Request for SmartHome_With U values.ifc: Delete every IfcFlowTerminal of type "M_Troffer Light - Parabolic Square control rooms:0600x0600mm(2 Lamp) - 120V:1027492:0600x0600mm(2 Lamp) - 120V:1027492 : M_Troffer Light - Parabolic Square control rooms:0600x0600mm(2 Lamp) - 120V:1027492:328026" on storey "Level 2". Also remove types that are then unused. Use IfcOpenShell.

First a look at what the model holds.

```python
import ifcopenshell
import ifcopenshell.util.element

model = ifcopenshell.open("SmartHome_With U values.ifc")
print(model.schema)
storey = next(s for s in model.by_type("IfcBuildingStorey") if s.Name == "Level 2")
terminals = [e for e in ifcopenshell.util.element.get_decomposition(storey) if e.is_a("IfcFlowTerminal")]
seen = {}
for e in terminals:
    element_type = ifcopenshell.util.element.get_type(e)
    name = element_type.Name if element_type not in (None, e) else None
    seen[name] = seen.get(name, 0) + 1
for name, count in sorted(seen.items(), key=str):
    print(count, "x", name)
```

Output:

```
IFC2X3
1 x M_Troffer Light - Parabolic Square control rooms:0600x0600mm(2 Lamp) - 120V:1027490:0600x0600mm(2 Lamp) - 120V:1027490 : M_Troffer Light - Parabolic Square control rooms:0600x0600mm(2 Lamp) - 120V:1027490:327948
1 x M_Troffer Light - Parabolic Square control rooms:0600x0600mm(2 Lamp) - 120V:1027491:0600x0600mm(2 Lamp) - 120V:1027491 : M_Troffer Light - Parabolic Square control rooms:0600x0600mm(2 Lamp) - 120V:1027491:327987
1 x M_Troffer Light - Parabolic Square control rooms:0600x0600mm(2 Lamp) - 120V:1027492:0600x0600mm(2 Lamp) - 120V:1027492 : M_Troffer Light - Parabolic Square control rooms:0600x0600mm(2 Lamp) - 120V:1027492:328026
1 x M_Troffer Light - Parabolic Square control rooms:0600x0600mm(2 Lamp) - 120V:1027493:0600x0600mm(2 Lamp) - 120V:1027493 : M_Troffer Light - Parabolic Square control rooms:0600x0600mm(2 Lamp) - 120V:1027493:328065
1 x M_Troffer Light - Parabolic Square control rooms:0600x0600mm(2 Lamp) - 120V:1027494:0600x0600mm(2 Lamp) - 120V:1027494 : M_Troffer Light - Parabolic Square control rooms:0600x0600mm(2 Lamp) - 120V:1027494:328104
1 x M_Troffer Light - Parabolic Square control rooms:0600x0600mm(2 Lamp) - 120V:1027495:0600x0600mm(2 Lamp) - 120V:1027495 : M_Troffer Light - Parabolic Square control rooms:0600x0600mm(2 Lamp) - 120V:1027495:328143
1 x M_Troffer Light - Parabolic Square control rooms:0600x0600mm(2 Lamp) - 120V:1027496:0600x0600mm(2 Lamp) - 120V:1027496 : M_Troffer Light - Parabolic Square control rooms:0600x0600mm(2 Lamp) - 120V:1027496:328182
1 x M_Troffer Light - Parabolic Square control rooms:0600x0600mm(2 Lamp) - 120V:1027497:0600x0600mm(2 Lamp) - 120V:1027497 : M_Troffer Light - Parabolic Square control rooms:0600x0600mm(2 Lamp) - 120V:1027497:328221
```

```python
import ifcopenshell
import ifcopenshell.api.root
import ifcopenshell.util.element

model = ifcopenshell.open("SmartHome_With U values.ifc")

storey = next(s for s in model.by_type("IfcBuildingStorey") if s.Name == "Level 2")
terminals = [e for e in ifcopenshell.util.element.get_decomposition(storey) if e.is_a("IfcFlowTerminal")]
targets = [e for e in terminals if (t := ifcopenshell.util.element.get_type(e)) not in (None, e) and t.Name == "M_Troffer Light - Parabolic Square control rooms:0600x0600mm(2 Lamp) - 120V:1027492:0600x0600mm(2 Lamp) - 120V:1027492 : M_Troffer Light - Parabolic Square control rooms:0600x0600mm(2 Lamp) - 120V:1027492:328026"]
types = {ifcopenshell.util.element.get_type(e) for e in targets} - {None, *targets}

for e in targets:
    ifcopenshell.api.root.remove_product(model, product=e)
print(len(targets), "removed")

unused = [t for t in types if not ifcopenshell.util.element.get_types(t)]
for t in unused:
    ifcopenshell.api.root.remove_product(model, product=t)
print(len(unused), "unused types removed")

model.write("SmartHome_With U values_v2.ifc")
```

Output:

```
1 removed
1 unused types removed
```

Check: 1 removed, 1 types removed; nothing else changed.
